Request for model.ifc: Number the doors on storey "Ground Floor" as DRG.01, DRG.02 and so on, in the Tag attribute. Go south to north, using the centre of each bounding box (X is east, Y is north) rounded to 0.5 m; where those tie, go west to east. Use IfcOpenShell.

First a look at what the model holds.

```python
import ifcopenshell
import ifcopenshell.util.element
import ifcopenshell.util.placement

model = ifcopenshell.open("model.ifc")
print(model.schema)
storey = next(s for s in model.by_type("IfcBuildingStorey") if s.Name == "Ground Floor")
doors = [e for e in ifcopenshell.util.element.get_decomposition(storey) if e.is_a("IfcDoor")]
for e in sorted(doors, key=lambda e: e.id()):
    origin = ifcopenshell.util.placement.get_local_placement(e.ObjectPlacement)[:3, 3]
    print(e.id(), e.Tag, e.Name, origin.round(2) + 0.0, sep=" | ")
```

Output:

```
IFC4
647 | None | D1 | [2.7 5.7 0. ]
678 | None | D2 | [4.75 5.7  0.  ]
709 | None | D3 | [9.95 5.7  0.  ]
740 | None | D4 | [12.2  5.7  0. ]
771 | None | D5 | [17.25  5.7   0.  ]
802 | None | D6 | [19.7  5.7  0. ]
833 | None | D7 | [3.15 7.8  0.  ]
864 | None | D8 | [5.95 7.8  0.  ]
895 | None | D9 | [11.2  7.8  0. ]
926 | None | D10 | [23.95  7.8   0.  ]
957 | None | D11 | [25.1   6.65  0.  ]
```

```python
import ifcopenshell
import ifcopenshell.geom
import ifcopenshell.util.element
import ifcopenshell.util.shape

model = ifcopenshell.open("model.ifc")
settings = ifcopenshell.geom.settings()
settings.set("use-world-coords", True)


def centre(element):
    shape = ifcopenshell.geom.create_shape(settings, element)
    return ifcopenshell.util.shape.get_bbox_centroid(shape.geometry)


storey = next(s for s in model.by_type("IfcBuildingStorey") if s.Name == "Ground Floor")
doors = [e for e in ifcopenshell.util.element.get_decomposition(storey) if e.is_a("IfcDoor")]

# Insertion points can sit at a corner or the storey origin, so sort by the geometry (in metres).
centres = {e: centre(e) for e in doors}
doors.sort(key=lambda e: (round(centres[e][1] / 0.5), centres[e][0]))

for i, e in enumerate(doors, start=1):
    number = f"DRG.{i:02d}"
    e.Tag = number
    print(e.id(), number)

model.write("model_rev.ifc")
```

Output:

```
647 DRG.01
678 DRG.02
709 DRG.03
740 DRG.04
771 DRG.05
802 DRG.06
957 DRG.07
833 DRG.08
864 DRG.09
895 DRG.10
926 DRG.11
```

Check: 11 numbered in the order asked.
